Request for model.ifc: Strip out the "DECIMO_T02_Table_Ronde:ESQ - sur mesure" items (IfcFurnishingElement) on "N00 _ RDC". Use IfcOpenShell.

First a look at what the model holds.

```python
import ifcopenshell
import ifcopenshell.util.element

model = ifcopenshell.open("model.ifc")
print(model.schema)
storey = next(s for s in model.by_type("IfcBuildingStorey") if s.Name == "N00 _ RDC")
furniture = [e for e in ifcopenshell.util.element.get_decomposition(storey) if e.is_a("IfcFurnishingElement")]
seen = {}
for e in furniture:
    element_type = ifcopenshell.util.element.get_type(e)
    name = element_type.Name if element_type not in (None, e) else None
    seen[name] = seen.get(name, 0) + 1
for name, count in sorted(seen.items(), key=str):
    print(count, "x", name)
```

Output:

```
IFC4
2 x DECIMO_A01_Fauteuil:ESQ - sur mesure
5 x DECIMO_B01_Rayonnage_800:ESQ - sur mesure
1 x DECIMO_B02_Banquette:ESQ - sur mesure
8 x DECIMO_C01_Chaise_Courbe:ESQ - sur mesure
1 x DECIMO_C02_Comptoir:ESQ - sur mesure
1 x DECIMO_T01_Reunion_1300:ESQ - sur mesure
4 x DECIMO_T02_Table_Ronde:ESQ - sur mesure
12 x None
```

```python
import ifcopenshell
import ifcopenshell.api.root
import ifcopenshell.util.element

model = ifcopenshell.open("model.ifc")

storey = next(s for s in model.by_type("IfcBuildingStorey") if s.Name == "N00 _ RDC")
furniture = [e for e in ifcopenshell.util.element.get_decomposition(storey) if e.is_a("IfcFurnishingElement")]
targets = [e for e in furniture if (t := ifcopenshell.util.element.get_type(e)) not in (None, e) and t.Name == "DECIMO_T02_Table_Ronde:ESQ - sur mesure"]

for e in targets:
    ifcopenshell.api.root.remove_product(model, product=e)
print(len(targets), "removed")

model.write("model_v2.ifc")
```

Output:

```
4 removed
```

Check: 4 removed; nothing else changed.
